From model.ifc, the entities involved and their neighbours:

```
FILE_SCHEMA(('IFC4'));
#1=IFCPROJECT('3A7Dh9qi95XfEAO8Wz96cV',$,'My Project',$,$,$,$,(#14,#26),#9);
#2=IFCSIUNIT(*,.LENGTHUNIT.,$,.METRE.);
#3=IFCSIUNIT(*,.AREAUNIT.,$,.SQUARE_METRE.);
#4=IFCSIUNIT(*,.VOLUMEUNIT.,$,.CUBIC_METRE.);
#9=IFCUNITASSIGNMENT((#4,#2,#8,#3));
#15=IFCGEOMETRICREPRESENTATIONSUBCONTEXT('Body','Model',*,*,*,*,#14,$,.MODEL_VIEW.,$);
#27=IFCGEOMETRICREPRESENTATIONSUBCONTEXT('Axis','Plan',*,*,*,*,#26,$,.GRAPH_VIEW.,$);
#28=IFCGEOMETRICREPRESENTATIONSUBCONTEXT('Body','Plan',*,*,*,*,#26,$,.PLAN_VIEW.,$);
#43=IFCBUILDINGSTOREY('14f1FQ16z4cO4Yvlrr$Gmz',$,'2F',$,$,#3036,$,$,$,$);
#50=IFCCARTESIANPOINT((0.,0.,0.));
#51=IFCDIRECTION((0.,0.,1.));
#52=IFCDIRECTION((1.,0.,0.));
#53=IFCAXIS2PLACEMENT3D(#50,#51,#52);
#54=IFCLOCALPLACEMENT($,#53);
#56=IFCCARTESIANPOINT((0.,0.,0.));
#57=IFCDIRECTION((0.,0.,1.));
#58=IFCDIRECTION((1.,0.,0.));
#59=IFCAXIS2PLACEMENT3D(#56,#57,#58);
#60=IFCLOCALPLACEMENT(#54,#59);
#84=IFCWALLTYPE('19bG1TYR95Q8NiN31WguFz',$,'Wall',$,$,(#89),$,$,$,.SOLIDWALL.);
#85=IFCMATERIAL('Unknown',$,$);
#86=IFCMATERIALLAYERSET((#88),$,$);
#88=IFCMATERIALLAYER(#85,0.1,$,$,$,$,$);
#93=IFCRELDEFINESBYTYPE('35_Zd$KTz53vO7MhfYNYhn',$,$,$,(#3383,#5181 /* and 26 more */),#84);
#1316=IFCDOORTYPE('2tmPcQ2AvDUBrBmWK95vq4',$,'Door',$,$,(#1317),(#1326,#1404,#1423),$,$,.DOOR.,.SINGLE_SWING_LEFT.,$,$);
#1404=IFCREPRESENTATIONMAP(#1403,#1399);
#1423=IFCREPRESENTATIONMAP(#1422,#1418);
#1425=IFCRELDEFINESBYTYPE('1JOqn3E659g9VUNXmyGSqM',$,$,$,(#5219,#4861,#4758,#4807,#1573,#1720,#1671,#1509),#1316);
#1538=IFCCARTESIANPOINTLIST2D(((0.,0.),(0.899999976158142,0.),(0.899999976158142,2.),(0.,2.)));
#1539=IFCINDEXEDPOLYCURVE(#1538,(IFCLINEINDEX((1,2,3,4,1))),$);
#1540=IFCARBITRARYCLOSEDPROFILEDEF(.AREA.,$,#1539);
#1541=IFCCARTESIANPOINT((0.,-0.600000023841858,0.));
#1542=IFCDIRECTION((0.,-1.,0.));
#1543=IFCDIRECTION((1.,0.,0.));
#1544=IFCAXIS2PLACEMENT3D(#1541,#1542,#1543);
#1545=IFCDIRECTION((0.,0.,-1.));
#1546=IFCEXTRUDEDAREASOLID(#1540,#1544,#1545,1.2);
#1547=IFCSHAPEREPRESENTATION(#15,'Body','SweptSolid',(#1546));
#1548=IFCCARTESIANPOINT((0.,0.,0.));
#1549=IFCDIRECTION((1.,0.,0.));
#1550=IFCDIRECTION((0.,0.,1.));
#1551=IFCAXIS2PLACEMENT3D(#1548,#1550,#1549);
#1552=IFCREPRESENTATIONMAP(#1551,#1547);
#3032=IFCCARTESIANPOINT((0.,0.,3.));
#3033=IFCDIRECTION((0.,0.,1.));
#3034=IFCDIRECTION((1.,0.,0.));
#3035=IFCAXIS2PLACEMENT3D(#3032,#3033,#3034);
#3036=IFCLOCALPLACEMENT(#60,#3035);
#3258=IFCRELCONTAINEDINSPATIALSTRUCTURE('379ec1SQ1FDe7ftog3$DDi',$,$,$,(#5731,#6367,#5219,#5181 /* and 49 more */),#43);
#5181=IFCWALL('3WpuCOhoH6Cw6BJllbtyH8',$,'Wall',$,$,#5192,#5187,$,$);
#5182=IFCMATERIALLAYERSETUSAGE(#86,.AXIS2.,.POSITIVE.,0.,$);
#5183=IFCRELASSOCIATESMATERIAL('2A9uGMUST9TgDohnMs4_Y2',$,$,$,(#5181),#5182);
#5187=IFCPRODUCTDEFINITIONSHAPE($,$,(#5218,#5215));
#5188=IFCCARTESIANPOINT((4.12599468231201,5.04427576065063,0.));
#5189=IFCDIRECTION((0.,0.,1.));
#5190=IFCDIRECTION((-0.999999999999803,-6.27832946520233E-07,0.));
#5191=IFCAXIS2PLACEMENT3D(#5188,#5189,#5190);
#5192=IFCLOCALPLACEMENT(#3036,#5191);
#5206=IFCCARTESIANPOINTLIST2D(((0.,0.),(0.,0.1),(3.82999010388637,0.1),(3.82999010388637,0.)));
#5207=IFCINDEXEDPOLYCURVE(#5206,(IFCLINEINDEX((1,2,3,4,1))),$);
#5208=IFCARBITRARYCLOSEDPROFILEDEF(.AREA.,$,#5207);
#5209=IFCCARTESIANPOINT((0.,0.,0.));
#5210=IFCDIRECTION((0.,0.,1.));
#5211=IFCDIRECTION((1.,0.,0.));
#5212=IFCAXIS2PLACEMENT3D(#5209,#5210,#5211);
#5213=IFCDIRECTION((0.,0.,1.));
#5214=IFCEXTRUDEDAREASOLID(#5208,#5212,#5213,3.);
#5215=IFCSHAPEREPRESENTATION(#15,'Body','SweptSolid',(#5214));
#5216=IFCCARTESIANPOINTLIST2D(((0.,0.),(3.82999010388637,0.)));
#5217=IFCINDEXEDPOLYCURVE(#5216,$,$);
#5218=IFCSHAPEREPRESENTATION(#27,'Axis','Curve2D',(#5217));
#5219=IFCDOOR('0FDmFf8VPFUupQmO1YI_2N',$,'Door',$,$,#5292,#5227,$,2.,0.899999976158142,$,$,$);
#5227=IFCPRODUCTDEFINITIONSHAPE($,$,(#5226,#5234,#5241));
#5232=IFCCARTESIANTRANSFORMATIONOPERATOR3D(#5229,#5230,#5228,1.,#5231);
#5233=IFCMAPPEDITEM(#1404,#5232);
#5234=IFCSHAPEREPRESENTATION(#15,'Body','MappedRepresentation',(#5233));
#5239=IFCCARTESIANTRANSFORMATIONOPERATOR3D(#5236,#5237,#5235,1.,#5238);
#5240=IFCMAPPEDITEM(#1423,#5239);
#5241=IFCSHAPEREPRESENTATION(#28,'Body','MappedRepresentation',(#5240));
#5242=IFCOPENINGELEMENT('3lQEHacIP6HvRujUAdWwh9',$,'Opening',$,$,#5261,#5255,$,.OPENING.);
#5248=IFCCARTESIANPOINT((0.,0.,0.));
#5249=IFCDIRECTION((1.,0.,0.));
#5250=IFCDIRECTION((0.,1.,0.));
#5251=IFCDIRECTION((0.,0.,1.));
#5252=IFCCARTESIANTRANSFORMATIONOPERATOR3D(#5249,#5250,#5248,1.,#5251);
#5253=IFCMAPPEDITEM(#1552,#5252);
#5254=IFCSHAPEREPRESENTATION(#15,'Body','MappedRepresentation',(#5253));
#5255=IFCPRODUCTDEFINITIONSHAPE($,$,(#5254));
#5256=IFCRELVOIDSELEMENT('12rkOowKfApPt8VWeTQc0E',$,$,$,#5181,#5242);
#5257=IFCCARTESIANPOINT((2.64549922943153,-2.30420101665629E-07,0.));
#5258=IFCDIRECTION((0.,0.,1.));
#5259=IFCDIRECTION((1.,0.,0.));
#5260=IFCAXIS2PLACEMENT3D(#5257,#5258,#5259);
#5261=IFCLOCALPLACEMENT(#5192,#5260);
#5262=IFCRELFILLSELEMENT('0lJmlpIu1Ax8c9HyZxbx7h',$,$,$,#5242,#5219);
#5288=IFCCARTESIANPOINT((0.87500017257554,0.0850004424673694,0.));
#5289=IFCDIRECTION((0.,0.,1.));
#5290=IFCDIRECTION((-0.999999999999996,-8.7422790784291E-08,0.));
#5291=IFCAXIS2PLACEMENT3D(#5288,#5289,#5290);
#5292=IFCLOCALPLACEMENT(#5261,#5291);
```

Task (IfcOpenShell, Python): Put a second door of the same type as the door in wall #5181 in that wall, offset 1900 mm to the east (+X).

```python
import ifcopenshell
import ifcopenshell.api.feature
import ifcopenshell.api.geometry
import ifcopenshell.api.root
import ifcopenshell.geom
import ifcopenshell.util.element
import ifcopenshell.util.placement
import ifcopenshell.util.shape

model = ifcopenshell.open("model.ifc")
settings = ifcopenshell.geom.settings()


def volume(element):
    """Net volume in cubic metres, openings subtracted."""
    shape = ifcopenshell.geom.create_shape(settings, element)
    return ifcopenshell.util.shape.get_volume(shape.geometry)


door = model.by_guid("0FDmFf8VPFUupQmO1YI_2N")
opening = door.FillsVoids[0].RelatingOpeningElement
wall = opening.VoidsElements[0].RelatingBuildingElement
before = volume(wall)
shift = ifcopenshell.util.placement.get_local_placement(wall.ObjectPlacement)[:3, 0] * -1.9

# copy_class copies the void relationship, type, container and properties, but no geometry.
new_opening = ifcopenshell.api.root.copy_class(model, product=opening)
new_opening.Representation = ifcopenshell.util.element.copy_deep(
    model, opening.Representation, exclude=["IfcGeometricRepresentationContext", "IfcRepresentationMap"]
)
new_door = ifcopenshell.api.root.copy_class(model, product=door)
new_door.Representation = ifcopenshell.util.element.copy_deep(
    model, door.Representation, exclude=["IfcGeometricRepresentationContext", "IfcRepresentationMap"]
)
ifcopenshell.api.feature.add_filling(model, opening=new_opening, element=new_door)

for old, new in ((opening, new_opening), (door, new_door)):
    matrix = ifcopenshell.util.placement.get_local_placement(old.ObjectPlacement)
    matrix[:3, 3] += shift
    ifcopenshell.api.geometry.edit_object_placement(model, product=new, matrix=matrix, is_si=False)

after = volume(wall)

print(f"wall volume {before:.3f} -> {after:.3f} m3")

model.write("model-out.ifc")
```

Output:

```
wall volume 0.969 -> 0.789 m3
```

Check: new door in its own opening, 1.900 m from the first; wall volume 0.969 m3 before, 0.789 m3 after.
